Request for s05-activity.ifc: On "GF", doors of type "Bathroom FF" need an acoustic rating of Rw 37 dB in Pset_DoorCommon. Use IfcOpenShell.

First a look at what the model holds.

```python
import ifcopenshell
import ifcopenshell.util.element

model = ifcopenshell.open("s05-activity.ifc")
print(model.schema)
storey = next(s for s in model.by_type("IfcBuildingStorey") if s.Name == "GF")
doors = [e for e in ifcopenshell.util.element.get_decomposition(storey) if e.is_a("IfcDoor")]
seen = {}
for e in doors:
    element_type = ifcopenshell.util.element.get_type(e)
    key = (element_type.Name if element_type != e and element_type else None, ifcopenshell.util.element.get_pset(e, "Pset_DoorCommon", "AcousticRating"))
    seen[key] = seen.get(key, 0) + 1
for (name, value), count in sorted(seen.items(), key=str):
    print(count, "x", name, "|", value)
```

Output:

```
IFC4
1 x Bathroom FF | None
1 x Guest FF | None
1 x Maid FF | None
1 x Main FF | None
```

```python
import ifcopenshell
import ifcopenshell.api.pset
import ifcopenshell.util.element

model = ifcopenshell.open("s05-activity.ifc")

storey = next(s for s in model.by_type("IfcBuildingStorey") if s.Name == "GF")
doors = [e for e in ifcopenshell.util.element.get_decomposition(storey) if e.is_a("IfcDoor")]

count = 0
for e in doors:
    element_type = ifcopenshell.util.element.get_type(e)
    if element_type in (None, e) or element_type.Name != "Bathroom FF":
        continue
    # add_pset returns the element's existing set when there is one.
    pset = ifcopenshell.api.pset.add_pset(model, product=e, name="Pset_DoorCommon")
    ifcopenshell.api.pset.edit_pset(model, pset=pset, properties={"AcousticRating": "Rw 37 dB"})
    count += 1

print(count, "doors updated")

model.write("s05-activity_v2.ifc")
```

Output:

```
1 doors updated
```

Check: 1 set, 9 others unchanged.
